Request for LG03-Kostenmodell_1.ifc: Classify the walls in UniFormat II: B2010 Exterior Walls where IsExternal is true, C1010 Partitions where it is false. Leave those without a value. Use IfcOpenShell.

First a look at what the model holds.

```python
import ifcopenshell
import ifcopenshell.util.element

model = ifcopenshell.open("LG03-Kostenmodell_1.ifc")
print(model.schema)
print("classifications:", [c.Name for c in model.by_type("IfcClassification")])
values = [ifcopenshell.util.element.get_pset(e, "Pset_WallCommon", "IsExternal") for e in model.by_type("IfcWall")]
for value in (True, False, None):
    print("IsExternal", value, values.count(value))
```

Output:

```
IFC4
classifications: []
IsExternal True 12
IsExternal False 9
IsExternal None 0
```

```python
import ifcopenshell
import ifcopenshell.api.classification
import ifcopenshell.util.element

model = ifcopenshell.open("LG03-Kostenmodell_1.ifc")

system = ifcopenshell.api.classification.add_classification(model, classification="UniFormat II")

walls = model.by_type("IfcWall")
external = {e: ifcopenshell.util.element.get_pset(e, "Pset_WallCommon", "IsExternal") for e in walls}
for flag, code, name in ((True, "B2010", "Exterior Walls"), (False, "C1010", "Partitions")):
    products = [e for e in walls if external[e] is flag]
    ifcopenshell.api.classification.add_reference(
        model, products=products, classification=system, identification=code, name=name
    )
    print(code, len(products))

model.write("LG03-Kostenmodell_1_edited.ifc")
```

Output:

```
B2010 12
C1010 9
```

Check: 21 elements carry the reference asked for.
